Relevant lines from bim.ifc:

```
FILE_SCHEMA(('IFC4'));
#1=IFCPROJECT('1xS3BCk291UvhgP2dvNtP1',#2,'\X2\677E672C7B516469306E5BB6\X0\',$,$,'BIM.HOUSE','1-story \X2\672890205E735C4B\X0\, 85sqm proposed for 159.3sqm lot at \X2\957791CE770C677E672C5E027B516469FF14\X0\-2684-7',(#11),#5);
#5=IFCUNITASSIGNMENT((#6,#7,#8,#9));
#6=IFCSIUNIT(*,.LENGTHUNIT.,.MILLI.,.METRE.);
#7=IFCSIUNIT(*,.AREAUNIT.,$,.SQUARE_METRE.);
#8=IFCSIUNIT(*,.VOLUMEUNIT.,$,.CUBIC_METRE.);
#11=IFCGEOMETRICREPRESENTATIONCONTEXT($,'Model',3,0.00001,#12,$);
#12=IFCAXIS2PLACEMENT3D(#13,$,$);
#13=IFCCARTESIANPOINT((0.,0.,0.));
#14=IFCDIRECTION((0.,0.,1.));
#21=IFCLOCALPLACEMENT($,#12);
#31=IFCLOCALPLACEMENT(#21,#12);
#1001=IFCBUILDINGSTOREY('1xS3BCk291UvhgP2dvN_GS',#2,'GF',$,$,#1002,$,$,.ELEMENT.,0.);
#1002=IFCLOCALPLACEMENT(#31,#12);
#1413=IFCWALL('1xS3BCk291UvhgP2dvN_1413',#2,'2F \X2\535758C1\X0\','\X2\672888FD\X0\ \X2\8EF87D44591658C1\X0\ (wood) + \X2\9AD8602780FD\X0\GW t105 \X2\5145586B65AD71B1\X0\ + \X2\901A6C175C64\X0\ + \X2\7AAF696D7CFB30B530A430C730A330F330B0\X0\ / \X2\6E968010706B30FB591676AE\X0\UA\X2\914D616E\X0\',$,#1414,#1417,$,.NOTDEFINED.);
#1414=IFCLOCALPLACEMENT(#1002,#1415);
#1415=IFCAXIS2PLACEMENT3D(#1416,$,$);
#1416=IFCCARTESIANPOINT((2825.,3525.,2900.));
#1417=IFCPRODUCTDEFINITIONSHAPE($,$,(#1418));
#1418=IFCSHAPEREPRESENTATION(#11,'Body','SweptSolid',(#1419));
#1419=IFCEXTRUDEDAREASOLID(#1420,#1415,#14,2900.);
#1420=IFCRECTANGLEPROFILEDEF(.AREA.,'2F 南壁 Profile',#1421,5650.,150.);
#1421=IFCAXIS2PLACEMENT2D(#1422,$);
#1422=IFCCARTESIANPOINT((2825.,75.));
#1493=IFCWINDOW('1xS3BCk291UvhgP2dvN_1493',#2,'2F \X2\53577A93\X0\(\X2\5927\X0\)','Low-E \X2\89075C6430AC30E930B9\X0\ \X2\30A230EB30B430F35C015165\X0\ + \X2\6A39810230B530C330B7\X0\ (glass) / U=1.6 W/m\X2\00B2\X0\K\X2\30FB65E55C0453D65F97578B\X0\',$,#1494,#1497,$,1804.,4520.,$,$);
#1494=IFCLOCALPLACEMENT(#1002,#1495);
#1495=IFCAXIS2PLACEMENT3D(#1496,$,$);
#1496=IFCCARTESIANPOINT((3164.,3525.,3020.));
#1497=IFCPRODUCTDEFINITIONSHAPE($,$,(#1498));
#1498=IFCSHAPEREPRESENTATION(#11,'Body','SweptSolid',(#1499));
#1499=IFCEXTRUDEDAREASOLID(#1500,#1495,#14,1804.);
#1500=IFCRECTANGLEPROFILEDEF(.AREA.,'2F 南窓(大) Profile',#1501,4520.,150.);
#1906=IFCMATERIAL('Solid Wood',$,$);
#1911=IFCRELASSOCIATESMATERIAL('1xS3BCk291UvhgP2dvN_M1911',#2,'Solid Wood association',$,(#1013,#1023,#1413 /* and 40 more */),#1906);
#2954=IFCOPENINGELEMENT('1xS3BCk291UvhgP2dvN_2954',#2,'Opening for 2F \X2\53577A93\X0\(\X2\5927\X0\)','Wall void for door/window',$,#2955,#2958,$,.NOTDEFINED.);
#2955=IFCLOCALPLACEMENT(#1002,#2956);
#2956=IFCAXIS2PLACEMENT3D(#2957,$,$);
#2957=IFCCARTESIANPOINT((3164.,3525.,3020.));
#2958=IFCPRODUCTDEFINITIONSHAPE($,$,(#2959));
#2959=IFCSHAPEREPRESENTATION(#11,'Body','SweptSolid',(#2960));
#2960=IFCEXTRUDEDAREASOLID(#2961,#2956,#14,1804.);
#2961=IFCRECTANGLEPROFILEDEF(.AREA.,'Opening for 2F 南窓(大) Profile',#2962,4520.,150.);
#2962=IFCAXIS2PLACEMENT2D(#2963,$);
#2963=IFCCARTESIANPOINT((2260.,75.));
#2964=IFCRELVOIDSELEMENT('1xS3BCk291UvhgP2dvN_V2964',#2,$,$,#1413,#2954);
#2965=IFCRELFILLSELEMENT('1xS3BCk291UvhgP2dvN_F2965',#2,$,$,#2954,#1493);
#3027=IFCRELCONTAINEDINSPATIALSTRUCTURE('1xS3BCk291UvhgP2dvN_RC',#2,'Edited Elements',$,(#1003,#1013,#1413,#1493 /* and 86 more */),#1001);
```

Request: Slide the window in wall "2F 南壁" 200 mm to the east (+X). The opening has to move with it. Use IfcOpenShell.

```python
import ifcopenshell
import ifcopenshell.api.geometry
import ifcopenshell.util.placement

model = ifcopenshell.open("bim.ifc")

window = model.by_id(1493)
opening = window.FillsVoids[0].RelatingOpeningElement
wall = opening.VoidsElements[0].RelatingBuildingElement

wall_matrix = ifcopenshell.util.placement.get_local_placement(wall.ObjectPlacement)
shift = wall_matrix[:3, 0] * 200.0
before = ifcopenshell.util.placement.get_local_placement(window.ObjectPlacement)[:3, 3].copy()

# The window is not placed relative to its opening, so move both.
for product in (opening, window):
    matrix = ifcopenshell.util.placement.get_local_placement(product.ObjectPlacement)
    matrix[:3, 3] += shift
    ifcopenshell.api.geometry.edit_object_placement(model, product=product, matrix=matrix, is_si=False)

after = ifcopenshell.util.placement.get_local_placement(window.ObjectPlacement)[:3, 3]
print("window moved by", (after - before).round(3) + 0.0)

model.write("bim-out.ifc")
```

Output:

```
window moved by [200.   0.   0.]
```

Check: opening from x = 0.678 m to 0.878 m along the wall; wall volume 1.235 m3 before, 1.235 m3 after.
